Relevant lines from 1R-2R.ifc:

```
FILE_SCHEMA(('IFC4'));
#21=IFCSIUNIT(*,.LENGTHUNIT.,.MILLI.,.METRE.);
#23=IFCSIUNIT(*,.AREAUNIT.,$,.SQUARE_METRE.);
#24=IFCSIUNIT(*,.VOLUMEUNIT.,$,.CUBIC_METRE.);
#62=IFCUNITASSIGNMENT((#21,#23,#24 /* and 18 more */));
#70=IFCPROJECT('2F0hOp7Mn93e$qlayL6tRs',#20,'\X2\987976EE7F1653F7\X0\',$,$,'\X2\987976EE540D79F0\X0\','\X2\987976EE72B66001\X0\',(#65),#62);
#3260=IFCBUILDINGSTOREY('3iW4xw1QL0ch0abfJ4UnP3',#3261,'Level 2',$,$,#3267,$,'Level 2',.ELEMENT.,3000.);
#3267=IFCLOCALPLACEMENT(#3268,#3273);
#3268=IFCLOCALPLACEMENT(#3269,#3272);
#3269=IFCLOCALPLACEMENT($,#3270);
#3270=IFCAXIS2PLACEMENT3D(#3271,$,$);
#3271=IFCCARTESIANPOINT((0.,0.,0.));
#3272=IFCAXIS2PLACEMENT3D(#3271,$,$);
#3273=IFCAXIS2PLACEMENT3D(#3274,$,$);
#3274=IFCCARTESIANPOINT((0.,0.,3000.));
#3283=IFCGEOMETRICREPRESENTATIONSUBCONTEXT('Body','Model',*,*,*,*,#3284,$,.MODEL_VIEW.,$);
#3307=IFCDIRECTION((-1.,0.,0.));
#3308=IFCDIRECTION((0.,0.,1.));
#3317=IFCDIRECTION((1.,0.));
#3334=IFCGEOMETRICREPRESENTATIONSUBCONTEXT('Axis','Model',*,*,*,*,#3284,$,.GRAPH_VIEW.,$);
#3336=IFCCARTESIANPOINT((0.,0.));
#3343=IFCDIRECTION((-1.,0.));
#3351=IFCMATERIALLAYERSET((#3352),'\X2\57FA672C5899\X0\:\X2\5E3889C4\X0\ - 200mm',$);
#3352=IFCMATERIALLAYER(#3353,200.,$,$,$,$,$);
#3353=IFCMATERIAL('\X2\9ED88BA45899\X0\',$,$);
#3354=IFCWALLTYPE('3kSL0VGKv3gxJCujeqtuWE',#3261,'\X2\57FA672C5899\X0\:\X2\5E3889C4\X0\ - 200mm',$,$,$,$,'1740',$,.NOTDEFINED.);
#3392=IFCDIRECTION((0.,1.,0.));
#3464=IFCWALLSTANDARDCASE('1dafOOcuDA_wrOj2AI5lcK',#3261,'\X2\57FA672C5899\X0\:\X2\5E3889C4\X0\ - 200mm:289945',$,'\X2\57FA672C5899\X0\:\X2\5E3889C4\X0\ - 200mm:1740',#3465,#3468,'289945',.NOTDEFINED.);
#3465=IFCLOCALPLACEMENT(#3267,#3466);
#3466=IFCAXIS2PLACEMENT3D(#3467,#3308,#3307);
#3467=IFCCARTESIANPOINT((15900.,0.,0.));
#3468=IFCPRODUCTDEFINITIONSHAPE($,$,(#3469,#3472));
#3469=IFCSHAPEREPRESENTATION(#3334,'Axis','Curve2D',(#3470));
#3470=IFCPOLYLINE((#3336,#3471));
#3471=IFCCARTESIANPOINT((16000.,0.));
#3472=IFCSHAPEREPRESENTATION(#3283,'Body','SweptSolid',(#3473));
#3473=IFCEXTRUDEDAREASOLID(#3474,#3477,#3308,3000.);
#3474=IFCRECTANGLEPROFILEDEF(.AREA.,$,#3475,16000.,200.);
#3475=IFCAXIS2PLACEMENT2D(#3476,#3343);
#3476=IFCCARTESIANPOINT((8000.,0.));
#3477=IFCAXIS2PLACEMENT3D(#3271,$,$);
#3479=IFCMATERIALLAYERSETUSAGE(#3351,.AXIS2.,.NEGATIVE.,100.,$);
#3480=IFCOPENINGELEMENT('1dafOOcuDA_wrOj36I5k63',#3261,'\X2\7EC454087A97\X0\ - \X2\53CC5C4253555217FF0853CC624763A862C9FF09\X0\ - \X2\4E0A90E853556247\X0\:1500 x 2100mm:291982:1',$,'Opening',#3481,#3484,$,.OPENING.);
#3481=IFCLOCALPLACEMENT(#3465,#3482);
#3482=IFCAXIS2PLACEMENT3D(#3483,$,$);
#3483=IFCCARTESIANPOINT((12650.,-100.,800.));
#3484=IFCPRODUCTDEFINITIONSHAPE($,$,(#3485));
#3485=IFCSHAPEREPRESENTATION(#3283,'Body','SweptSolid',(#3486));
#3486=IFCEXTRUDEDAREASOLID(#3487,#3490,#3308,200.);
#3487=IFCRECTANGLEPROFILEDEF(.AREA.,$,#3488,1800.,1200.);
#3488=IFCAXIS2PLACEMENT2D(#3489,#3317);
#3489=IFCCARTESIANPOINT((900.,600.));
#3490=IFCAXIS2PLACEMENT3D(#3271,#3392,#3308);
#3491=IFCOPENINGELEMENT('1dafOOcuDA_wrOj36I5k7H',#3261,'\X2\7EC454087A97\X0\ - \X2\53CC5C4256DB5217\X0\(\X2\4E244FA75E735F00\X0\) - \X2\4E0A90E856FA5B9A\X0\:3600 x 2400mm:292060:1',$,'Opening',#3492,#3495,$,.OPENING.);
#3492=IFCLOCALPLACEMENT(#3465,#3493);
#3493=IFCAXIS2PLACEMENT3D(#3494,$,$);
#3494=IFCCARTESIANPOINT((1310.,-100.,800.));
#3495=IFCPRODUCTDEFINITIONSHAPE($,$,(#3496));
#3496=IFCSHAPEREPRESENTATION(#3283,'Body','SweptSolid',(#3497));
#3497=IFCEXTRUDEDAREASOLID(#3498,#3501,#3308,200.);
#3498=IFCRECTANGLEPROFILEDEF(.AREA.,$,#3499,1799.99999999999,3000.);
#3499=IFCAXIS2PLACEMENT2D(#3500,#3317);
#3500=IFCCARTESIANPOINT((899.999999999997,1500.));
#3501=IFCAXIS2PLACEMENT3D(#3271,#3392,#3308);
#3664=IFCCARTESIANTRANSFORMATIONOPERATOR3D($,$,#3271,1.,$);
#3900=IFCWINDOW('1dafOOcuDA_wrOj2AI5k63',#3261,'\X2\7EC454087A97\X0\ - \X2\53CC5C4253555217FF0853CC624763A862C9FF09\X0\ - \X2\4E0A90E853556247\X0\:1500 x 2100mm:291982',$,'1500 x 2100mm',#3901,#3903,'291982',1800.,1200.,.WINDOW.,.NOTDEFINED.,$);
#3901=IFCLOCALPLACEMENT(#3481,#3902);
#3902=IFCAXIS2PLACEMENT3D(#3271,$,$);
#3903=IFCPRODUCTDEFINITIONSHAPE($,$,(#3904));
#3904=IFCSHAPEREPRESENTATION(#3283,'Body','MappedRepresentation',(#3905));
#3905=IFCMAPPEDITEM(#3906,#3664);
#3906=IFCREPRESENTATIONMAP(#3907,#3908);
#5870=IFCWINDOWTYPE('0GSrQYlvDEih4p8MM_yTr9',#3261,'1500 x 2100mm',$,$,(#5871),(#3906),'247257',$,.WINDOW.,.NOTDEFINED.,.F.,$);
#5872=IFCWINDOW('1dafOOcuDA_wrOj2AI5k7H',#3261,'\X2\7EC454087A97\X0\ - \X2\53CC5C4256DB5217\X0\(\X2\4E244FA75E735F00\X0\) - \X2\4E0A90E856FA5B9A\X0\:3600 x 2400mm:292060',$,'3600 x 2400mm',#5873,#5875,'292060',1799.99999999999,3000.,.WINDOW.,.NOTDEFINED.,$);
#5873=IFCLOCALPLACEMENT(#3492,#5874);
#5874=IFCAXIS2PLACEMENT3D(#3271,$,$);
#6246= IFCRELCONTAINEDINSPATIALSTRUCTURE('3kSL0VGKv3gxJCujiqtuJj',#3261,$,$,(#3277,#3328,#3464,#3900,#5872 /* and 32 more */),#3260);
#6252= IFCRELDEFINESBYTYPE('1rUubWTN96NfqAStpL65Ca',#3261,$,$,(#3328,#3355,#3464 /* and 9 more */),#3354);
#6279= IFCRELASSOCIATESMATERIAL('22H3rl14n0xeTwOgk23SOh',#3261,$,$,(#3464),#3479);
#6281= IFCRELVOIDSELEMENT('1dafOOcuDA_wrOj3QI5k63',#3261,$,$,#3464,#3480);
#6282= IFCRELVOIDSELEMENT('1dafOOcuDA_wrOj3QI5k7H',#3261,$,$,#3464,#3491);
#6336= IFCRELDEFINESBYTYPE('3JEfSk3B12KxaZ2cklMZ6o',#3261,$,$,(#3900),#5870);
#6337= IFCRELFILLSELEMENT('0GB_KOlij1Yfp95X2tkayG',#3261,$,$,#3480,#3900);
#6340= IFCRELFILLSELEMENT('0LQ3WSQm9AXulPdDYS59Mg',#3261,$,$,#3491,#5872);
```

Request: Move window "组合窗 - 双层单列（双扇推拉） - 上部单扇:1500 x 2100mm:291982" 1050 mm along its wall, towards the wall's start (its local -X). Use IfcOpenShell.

```python
import ifcopenshell
import ifcopenshell.api.geometry
import ifcopenshell.util.placement

model = ifcopenshell.open("1R-2R.ifc")

window = model.by_id(3900)
opening = window.FillsVoids[0].RelatingOpeningElement
wall = opening.VoidsElements[0].RelatingBuildingElement

wall_matrix = ifcopenshell.util.placement.get_local_placement(wall.ObjectPlacement)
shift = wall_matrix[:3, 0] * -1050.0
before = ifcopenshell.util.placement.get_local_placement(window.ObjectPlacement)[:3, 3].copy()

# The window is placed relative to its opening, so it follows when the opening moves.
matrix = ifcopenshell.util.placement.get_local_placement(opening.ObjectPlacement)
matrix[:3, 3] += shift
ifcopenshell.api.geometry.edit_object_placement(
    model, product=opening, matrix=matrix, is_si=False, should_transform_children=True
)

after = ifcopenshell.util.placement.get_local_placement(window.ObjectPlacement)[:3, 3]
print("window moved by", (after - before).round(3) + 0.0)

model.write("1R-2R_edited.ifc")
```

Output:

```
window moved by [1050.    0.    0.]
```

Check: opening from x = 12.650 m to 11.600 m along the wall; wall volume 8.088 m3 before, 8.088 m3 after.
